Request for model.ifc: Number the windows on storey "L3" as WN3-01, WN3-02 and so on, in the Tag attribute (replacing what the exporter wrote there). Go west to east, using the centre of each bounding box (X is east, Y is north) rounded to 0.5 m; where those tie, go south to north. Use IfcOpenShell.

First a look at what the model holds.

```python
import ifcopenshell
import ifcopenshell.util.element
import ifcopenshell.util.placement

model = ifcopenshell.open("model.ifc")
print(model.schema)
storey = next(s for s in model.by_type("IfcBuildingStorey") if s.Name == "L3")
windows = [e for e in ifcopenshell.util.element.get_decomposition(storey) if e.is_a("IfcWindow")]
for e in sorted(windows, key=lambda e: e.id()):
    origin = ifcopenshell.util.placement.get_local_placement(e.ObjectPlacement)[:3, 3]
    print(e.id(), e.Tag, e.Name, origin.round(2) + 0.0, sep=" | ")
```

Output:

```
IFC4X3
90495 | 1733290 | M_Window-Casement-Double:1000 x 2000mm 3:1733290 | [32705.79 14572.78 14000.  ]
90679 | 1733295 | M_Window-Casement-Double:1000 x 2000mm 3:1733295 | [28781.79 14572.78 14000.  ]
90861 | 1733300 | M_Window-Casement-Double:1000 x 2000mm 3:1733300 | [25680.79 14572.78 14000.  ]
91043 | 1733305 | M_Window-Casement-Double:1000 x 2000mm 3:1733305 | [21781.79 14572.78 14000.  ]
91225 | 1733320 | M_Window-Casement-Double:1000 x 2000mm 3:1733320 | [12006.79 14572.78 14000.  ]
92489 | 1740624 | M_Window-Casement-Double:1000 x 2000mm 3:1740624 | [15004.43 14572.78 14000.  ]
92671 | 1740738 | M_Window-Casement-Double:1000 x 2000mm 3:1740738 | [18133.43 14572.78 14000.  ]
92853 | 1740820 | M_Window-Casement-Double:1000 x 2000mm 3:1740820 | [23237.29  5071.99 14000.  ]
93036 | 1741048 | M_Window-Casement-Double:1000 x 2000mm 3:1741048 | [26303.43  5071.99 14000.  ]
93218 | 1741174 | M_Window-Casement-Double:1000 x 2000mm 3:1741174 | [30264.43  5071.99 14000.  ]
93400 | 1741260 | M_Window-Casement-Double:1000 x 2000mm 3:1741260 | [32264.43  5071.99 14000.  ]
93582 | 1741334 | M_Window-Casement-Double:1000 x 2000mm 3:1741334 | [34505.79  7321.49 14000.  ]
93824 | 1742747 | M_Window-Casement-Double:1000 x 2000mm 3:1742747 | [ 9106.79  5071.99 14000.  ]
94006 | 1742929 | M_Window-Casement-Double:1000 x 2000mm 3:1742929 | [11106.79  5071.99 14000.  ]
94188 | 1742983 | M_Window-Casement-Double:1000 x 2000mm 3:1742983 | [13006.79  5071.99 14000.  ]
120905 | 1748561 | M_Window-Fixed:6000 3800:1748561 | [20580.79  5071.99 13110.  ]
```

```python
import ifcopenshell
import ifcopenshell.geom
import ifcopenshell.util.element
import ifcopenshell.util.shape

model = ifcopenshell.open("model.ifc")
settings = ifcopenshell.geom.settings()
settings.set("use-world-coords", True)


def centre(element):
    shape = ifcopenshell.geom.create_shape(settings, element)
    return ifcopenshell.util.shape.get_bbox_centroid(shape.geometry)


storey = next(s for s in model.by_type("IfcBuildingStorey") if s.Name == "L3")
windows = [e for e in ifcopenshell.util.element.get_decomposition(storey) if e.is_a("IfcWindow")]

# Insertion points can sit at a corner or the storey origin, so sort by the geometry (in metres).
centres = {e: centre(e) for e in windows}
windows.sort(key=lambda e: (round(centres[e][0] / 0.5), centres[e][1]))

for i, e in enumerate(windows, start=1):
    number = f"WN3-{i:02d}"
    e.Tag = number
    print(e.id(), number)

model.write("model-out.ifc")
```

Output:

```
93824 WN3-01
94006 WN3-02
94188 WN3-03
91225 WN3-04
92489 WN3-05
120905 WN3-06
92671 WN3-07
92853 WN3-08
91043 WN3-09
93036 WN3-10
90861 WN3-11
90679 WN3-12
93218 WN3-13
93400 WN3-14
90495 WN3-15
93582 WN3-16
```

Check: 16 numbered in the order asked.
